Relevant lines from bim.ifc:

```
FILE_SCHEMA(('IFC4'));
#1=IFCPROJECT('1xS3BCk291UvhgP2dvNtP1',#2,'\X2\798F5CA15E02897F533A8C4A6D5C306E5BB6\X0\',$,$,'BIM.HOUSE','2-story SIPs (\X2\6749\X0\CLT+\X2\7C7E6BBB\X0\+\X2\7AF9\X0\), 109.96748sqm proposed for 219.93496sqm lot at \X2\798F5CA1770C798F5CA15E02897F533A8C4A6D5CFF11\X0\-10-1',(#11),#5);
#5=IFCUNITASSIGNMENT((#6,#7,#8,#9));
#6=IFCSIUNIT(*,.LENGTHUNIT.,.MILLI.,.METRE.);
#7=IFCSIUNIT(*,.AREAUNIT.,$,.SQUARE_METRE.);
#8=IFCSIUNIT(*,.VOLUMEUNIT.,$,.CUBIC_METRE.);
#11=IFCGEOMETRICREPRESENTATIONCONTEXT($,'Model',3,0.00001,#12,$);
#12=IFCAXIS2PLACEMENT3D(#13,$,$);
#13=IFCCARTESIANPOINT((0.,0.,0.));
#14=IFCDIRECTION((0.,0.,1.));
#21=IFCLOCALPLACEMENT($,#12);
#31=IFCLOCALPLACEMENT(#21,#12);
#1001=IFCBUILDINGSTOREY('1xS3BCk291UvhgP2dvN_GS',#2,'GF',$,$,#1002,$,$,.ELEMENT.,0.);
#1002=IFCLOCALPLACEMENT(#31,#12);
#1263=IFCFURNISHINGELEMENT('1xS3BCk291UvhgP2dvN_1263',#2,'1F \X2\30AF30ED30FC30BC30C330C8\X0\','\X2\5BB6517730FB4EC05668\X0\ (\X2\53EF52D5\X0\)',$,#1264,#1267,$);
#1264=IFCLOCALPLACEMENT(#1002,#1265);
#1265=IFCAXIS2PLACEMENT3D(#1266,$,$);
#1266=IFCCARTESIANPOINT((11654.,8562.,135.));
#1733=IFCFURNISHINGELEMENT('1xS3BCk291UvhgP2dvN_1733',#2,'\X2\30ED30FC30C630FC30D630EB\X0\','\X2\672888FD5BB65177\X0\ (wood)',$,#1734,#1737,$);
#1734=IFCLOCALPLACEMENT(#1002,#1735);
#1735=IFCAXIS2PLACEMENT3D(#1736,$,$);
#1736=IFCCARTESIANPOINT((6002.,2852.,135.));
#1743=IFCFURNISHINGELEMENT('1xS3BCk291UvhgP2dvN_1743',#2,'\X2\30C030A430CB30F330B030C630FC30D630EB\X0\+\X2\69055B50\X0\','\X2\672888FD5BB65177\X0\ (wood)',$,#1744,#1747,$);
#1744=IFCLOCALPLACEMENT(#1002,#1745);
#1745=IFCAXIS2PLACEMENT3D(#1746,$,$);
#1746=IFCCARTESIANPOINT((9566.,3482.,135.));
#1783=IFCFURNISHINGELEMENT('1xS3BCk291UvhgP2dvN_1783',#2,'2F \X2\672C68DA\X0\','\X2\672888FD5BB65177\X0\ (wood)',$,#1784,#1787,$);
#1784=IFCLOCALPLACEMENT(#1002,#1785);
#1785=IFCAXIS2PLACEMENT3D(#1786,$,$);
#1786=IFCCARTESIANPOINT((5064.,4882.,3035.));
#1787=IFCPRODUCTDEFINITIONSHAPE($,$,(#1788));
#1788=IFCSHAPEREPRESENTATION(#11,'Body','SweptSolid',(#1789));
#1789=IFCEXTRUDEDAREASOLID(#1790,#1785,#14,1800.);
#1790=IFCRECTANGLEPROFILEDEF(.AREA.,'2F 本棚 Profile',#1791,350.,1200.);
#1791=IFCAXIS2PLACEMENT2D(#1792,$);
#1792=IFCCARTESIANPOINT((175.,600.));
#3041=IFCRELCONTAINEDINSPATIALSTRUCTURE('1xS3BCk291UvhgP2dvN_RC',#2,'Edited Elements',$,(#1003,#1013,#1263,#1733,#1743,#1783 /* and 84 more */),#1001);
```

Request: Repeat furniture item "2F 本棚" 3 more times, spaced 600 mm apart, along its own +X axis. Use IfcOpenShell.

```python
import ifcopenshell
import ifcopenshell.api.geometry
import ifcopenshell.api.root
import ifcopenshell.util.element
import ifcopenshell.util.placement
import ifcopenshell.util.unit

model = ifcopenshell.open("bim.ifc")
unit_scale = ifcopenshell.util.unit.calculate_unit_scale(model)


def reuse_history(source, copy):
    """copy_class also copies each property set's owner history, people and application; keep the originals."""
    for rel in copy.IsDefinedBy:
        if rel.is_a("IfcRelDefinesByProperties") and (history := rel.RelatingPropertyDefinition.OwnerHistory):
            rel.RelatingPropertyDefinition.OwnerHistory = source.OwnerHistory
            ifcopenshell.util.element.remove_deep2(model, history)


source = model.by_guid("1xS3BCk291UvhgP2dvN_1783")
base = ifcopenshell.util.placement.get_local_placement(source.ObjectPlacement)
step = base[:3, 0] * 0.6 / unit_scale

for i in range(1, 4):
    copy = ifcopenshell.api.root.copy_class(model, product=source)
    copy.Representation = ifcopenshell.util.element.copy_deep(
        model, source.Representation, exclude=["IfcGeometricRepresentationContext", "IfcRepresentationMap"]
    )
    reuse_history(source, copy)
    matrix = base.copy()
    matrix[:3, 3] += i * step
    print("added at", matrix[:3, 3].round(3) + 0.0)
    ifcopenshell.api.geometry.edit_object_placement(model, product=copy, matrix=matrix, is_si=False)

model.write("bim_rev.ifc")
```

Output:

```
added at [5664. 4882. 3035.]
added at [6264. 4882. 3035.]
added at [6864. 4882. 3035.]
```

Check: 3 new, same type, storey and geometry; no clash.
